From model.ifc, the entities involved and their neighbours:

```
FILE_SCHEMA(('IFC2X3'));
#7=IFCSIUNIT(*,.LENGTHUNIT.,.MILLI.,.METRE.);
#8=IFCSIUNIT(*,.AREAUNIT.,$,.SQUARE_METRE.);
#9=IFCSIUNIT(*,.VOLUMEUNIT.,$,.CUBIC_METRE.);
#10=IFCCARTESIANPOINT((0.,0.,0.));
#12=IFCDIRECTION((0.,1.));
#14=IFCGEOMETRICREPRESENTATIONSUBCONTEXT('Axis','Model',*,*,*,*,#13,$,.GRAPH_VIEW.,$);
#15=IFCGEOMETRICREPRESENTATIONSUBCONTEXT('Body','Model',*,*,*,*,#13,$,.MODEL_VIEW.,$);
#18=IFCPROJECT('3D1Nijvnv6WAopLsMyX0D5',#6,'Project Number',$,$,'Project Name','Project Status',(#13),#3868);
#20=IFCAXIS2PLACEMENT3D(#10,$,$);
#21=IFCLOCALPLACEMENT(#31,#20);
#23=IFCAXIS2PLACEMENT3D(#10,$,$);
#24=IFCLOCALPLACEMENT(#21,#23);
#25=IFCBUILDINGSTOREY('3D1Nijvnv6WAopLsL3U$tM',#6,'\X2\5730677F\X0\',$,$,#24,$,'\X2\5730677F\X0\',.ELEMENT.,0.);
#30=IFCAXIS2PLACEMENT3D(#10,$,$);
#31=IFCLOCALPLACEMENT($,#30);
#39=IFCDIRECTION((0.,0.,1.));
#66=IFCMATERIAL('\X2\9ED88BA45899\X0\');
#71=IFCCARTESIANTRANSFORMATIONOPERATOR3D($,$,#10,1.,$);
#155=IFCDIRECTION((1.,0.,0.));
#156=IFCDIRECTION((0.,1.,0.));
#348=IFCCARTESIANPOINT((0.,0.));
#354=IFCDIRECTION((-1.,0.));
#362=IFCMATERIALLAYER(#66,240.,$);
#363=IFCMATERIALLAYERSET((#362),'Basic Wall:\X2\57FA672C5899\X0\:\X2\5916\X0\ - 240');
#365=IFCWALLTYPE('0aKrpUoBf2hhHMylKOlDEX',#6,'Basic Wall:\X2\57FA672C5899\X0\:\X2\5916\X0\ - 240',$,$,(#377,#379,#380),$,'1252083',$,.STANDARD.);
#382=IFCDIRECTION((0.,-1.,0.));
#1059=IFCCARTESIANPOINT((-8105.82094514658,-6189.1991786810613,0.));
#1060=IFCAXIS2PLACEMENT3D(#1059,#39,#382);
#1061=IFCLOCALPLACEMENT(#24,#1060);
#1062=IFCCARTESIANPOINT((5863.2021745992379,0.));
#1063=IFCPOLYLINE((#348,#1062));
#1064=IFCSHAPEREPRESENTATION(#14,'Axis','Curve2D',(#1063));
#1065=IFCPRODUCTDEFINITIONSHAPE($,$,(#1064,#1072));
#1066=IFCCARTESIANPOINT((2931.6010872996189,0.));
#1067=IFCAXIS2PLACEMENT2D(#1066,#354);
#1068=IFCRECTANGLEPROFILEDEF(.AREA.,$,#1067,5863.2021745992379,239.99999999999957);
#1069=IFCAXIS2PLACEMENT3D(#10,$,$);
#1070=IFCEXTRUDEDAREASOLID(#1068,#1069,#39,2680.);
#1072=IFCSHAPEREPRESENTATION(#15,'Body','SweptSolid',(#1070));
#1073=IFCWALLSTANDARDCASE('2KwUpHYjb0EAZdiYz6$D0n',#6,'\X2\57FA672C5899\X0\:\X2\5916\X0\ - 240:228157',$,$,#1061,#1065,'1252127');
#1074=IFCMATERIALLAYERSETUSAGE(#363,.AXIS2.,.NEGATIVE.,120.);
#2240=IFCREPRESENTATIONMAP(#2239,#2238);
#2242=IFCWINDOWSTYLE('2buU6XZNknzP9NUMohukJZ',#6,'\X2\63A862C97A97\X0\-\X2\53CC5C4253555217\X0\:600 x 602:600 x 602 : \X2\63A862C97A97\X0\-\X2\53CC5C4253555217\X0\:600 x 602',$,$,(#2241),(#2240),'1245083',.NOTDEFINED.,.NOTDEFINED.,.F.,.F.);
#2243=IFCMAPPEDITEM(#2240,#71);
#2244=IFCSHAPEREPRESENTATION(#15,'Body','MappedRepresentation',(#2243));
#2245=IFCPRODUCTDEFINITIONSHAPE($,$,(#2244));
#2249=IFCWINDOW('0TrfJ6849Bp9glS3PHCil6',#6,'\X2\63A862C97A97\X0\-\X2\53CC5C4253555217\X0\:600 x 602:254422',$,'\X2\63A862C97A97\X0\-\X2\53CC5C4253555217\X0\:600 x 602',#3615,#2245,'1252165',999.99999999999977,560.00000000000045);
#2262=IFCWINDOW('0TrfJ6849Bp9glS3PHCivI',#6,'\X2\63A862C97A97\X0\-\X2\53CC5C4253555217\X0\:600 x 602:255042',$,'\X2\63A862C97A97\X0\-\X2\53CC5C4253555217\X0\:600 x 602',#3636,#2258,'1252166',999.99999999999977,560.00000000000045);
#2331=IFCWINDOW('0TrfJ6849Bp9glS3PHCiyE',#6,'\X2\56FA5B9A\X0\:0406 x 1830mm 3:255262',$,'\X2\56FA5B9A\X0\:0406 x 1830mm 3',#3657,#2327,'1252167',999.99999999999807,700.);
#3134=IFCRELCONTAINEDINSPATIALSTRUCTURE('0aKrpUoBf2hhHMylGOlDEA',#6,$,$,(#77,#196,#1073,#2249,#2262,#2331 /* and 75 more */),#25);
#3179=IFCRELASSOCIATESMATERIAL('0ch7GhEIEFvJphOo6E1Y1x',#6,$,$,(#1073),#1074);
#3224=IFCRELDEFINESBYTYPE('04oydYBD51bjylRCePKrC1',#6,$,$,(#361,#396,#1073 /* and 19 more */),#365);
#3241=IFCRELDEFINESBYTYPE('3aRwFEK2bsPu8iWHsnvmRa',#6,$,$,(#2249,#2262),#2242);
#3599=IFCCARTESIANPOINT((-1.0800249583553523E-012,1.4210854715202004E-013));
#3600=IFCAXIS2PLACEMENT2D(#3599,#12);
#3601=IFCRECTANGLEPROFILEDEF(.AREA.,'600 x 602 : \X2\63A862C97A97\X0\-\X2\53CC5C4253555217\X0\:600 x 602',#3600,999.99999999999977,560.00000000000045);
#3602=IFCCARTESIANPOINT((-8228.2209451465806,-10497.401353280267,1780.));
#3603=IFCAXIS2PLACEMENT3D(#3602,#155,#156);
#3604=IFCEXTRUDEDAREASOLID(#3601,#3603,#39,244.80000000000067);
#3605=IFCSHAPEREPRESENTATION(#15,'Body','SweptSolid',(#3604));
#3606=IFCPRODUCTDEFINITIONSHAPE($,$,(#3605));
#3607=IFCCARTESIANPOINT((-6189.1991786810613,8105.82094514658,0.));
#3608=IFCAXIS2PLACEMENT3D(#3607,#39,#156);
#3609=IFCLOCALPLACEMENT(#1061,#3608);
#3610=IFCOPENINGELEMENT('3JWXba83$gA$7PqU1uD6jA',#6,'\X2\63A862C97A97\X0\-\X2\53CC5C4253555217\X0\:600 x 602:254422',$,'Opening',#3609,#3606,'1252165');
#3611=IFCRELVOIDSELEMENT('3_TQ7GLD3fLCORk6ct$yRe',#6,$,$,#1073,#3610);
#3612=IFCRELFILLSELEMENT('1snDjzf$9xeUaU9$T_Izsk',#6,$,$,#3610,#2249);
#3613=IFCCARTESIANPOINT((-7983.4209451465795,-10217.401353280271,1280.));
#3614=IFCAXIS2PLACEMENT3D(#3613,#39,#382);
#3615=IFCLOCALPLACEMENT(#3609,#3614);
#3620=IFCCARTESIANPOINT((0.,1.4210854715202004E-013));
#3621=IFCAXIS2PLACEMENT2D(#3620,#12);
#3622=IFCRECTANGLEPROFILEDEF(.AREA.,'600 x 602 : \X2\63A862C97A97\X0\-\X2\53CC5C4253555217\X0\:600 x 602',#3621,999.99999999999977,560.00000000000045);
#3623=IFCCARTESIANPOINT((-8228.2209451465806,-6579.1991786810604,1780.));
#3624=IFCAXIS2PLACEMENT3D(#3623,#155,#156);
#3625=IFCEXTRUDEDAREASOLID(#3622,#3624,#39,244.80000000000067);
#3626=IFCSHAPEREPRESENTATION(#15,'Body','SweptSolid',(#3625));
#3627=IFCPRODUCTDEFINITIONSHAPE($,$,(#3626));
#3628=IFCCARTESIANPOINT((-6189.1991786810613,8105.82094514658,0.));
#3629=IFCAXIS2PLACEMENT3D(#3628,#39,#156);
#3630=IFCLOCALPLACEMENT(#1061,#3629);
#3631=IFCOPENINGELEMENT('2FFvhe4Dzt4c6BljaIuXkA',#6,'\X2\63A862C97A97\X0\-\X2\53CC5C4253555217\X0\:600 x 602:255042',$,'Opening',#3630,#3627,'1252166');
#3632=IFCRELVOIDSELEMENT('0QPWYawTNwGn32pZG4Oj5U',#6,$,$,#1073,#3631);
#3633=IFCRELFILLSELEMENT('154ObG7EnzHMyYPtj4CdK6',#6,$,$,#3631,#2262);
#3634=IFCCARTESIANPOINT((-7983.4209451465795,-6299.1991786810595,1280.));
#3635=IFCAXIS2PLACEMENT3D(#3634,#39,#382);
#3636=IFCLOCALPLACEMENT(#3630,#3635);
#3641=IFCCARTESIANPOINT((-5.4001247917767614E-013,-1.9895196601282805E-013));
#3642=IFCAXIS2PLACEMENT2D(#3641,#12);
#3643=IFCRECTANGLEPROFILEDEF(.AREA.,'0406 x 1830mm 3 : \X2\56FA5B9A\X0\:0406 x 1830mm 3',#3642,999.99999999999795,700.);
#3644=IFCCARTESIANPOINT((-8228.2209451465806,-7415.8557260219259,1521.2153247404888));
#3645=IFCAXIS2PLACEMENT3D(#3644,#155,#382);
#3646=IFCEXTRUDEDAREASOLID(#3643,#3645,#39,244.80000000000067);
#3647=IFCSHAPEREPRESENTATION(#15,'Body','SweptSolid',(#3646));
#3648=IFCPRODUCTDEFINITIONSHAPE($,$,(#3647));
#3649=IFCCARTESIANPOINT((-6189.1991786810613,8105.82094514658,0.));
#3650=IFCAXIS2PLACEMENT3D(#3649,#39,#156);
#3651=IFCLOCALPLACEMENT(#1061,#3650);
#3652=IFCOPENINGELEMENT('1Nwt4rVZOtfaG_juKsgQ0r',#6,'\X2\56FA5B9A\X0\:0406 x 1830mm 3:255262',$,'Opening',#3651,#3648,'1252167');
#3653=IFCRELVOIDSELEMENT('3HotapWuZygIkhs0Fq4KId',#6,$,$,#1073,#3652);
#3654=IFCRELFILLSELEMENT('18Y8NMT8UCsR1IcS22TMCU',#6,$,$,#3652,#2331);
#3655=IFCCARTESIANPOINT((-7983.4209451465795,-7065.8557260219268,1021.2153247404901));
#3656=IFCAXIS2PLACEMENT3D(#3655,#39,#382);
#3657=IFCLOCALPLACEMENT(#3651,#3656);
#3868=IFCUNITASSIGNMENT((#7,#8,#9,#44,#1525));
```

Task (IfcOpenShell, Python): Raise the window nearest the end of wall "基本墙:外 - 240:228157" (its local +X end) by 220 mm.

```python
import numpy as np
import ifcopenshell
import ifcopenshell.api.geometry
import ifcopenshell.util.placement
import ifcopenshell.util.unit

model = ifcopenshell.open("model.ifc")
unit_scale = ifcopenshell.util.unit.calculate_unit_scale(model)

window = model.by_guid("0TrfJ6849Bp9glS3PHCil6")
opening = window.FillsVoids[0].RelatingOpeningElement
dz = 220.0

shift = np.array([0.0, 0.0, dz])
# The window is placed relative to its opening, so it follows when the opening moves.
matrix = ifcopenshell.util.placement.get_local_placement(opening.ObjectPlacement)
matrix[:3, 3] += shift
ifcopenshell.api.geometry.edit_object_placement(
    model, product=opening, matrix=matrix, is_si=False, should_transform_children=True
)

print(f"moved by {dz * unit_scale:+.3f} m")

model.write("model_edited.ifc")
```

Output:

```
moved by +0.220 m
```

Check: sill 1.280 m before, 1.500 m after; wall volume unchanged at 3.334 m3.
